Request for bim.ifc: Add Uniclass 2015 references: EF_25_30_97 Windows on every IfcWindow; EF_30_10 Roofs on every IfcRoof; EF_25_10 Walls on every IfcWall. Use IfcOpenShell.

First a look at what the model holds.

```python
import ifcopenshell

model = ifcopenshell.open("bim.ifc")
print(model.schema)
print("classifications:", [c.Name for c in model.by_type("IfcClassification")])
for ifc_class in ("IfcDoor", "IfcRoof", "IfcStair", "IfcWall", "IfcWindow"):
    print(ifc_class, len(model.by_type(ifc_class)))
```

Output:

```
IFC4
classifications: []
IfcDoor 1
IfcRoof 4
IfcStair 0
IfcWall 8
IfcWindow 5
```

```python
import ifcopenshell
import ifcopenshell.api.classification

model = ifcopenshell.open("bim.ifc")

system = ifcopenshell.api.classification.add_classification(model, classification="Uniclass 2015")

codes = {
    "IfcWindow": ("EF_25_30_97", "Windows"),
    "IfcRoof": ("EF_30_10", "Roofs"),
    "IfcWall": ("EF_25_10", "Walls"),
}
for ifc_class, (code, name) in codes.items():
    products = model.by_type(ifc_class)
    ifcopenshell.api.classification.add_reference(
        model, products=products, classification=system, identification=code, name=name
    )
    print(code, len(products))

model.write("bim-out.ifc")
```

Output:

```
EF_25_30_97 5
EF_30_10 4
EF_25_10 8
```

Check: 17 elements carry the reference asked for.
